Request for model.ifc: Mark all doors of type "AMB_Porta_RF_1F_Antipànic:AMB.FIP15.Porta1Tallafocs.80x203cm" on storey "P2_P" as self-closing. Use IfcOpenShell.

First a look at what the model holds.

```python
import ifcopenshell
import ifcopenshell.util.element

model = ifcopenshell.open("model.ifc")
print(model.schema)
storey = next(s for s in model.by_type("IfcBuildingStorey") if s.Name == "P2_P")
doors = [e for e in ifcopenshell.util.element.get_decomposition(storey) if e.is_a("IfcDoor")]
seen = {}
for e in doors:
    element_type = ifcopenshell.util.element.get_type(e)
    key = (element_type.Name if element_type != e and element_type else None, ifcopenshell.util.element.get_pset(e, "Pset_DoorCommon", "SelfClosing"))
    seen[key] = seen.get(key, 0) + 1
for (name, value), count in sorted(seen.items(), key=str):
    print(count, "x", name, "|", value)
```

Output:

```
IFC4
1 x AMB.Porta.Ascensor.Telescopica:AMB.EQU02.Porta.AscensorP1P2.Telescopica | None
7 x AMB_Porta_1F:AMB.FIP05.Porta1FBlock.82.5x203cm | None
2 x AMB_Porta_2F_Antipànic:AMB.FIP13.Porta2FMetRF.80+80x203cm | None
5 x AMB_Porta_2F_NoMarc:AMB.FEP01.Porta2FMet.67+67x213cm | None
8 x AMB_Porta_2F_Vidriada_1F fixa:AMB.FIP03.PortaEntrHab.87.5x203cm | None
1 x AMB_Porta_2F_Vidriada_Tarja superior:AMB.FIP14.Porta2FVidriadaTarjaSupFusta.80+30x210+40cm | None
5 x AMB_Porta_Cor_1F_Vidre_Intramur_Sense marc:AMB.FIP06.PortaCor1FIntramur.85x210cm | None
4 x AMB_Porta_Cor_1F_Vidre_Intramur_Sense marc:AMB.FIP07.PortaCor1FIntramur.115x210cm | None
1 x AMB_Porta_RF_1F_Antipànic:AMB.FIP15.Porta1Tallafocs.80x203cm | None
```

```python
import ifcopenshell
import ifcopenshell.api.pset
import ifcopenshell.util.element

model = ifcopenshell.open("model.ifc")

storey = next(s for s in model.by_type("IfcBuildingStorey") if s.Name == "P2_P")
doors = [e for e in ifcopenshell.util.element.get_decomposition(storey) if e.is_a("IfcDoor")]

count = 0
for e in doors:
    element_type = ifcopenshell.util.element.get_type(e)
    if element_type in (None, e) or element_type.Name != "AMB_Porta_RF_1F_Antipànic:AMB.FIP15.Porta1Tallafocs.80x203cm":
        continue
    # add_pset returns the element's existing set when there is one.
    pset = ifcopenshell.api.pset.add_pset(model, product=e, name="Pset_DoorCommon")
    ifcopenshell.api.pset.edit_pset(model, pset=pset, properties={"SelfClosing": True})
    count += 1

print(count, "doors updated")

model.write("model_edited.ifc")
```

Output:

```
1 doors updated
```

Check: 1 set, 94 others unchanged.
